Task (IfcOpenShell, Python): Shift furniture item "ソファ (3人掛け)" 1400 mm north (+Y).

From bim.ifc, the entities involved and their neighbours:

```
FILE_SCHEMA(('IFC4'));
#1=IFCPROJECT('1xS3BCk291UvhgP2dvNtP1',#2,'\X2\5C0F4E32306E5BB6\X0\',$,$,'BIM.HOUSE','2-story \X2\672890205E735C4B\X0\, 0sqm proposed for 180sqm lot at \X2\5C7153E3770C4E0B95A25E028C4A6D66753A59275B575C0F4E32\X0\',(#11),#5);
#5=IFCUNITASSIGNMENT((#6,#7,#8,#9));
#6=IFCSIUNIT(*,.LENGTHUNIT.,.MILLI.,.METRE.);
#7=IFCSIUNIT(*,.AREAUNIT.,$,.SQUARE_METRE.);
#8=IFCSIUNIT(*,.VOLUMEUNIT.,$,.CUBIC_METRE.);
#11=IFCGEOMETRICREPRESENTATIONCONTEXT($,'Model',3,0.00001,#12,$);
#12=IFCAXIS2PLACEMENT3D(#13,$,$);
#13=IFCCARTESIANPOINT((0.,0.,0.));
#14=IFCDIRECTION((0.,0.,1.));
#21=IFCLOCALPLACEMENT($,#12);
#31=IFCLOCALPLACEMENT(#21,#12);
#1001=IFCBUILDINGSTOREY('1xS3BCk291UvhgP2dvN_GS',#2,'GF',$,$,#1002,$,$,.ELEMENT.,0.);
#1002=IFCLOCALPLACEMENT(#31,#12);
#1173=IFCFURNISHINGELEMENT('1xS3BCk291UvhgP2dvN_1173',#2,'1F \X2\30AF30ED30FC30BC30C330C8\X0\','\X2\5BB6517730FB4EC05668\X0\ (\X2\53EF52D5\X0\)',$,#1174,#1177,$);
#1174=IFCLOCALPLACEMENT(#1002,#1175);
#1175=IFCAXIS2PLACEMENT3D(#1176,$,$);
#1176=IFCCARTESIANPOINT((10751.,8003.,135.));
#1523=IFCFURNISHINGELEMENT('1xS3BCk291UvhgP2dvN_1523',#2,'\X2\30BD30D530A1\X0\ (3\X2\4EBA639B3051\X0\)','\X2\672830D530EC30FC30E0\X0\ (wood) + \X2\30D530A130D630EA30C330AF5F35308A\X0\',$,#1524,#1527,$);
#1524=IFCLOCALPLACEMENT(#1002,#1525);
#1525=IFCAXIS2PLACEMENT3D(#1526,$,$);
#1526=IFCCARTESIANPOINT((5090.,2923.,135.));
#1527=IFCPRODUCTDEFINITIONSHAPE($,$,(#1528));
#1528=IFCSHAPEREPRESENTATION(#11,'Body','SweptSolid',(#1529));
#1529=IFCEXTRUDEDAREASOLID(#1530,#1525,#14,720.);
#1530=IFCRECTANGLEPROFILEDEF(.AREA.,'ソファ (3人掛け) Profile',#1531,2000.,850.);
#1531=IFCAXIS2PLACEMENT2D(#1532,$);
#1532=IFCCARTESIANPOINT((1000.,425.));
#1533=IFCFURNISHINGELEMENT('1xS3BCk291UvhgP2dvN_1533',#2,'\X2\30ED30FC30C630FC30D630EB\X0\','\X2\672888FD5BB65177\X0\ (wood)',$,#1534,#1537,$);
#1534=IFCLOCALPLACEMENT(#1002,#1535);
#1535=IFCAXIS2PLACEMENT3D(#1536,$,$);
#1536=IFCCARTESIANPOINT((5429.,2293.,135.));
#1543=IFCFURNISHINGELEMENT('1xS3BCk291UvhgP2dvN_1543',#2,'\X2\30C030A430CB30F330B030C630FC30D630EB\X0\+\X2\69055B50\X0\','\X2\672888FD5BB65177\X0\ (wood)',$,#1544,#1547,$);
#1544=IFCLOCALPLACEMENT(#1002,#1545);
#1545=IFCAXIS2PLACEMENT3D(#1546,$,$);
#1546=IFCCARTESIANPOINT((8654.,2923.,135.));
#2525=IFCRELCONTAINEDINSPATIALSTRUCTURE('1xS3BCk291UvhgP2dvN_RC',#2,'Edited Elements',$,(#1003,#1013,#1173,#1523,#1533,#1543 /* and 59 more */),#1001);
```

```python
import ifcopenshell
import ifcopenshell.api.geometry
import ifcopenshell.util.placement
import ifcopenshell.util.unit

model = ifcopenshell.open("bim.ifc")
unit_scale = ifcopenshell.util.unit.calculate_unit_scale(model)

item = model.by_id(1523)
matrix = ifcopenshell.util.placement.get_local_placement(item.ObjectPlacement)
matrix[1, 3] += 1.4 / unit_scale
ifcopenshell.api.geometry.edit_object_placement(model, product=item, matrix=matrix, is_si=False)

print(ifcopenshell.util.placement.get_local_placement(item.ObjectPlacement).round(3) + 0.0)

model.write("bim_v2.ifc")
```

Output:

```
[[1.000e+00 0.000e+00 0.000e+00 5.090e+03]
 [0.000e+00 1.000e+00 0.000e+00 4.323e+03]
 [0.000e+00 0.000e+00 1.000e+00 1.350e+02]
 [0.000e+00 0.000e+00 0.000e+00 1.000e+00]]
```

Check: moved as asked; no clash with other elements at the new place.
